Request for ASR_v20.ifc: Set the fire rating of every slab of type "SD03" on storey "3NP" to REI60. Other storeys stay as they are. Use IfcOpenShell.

First a look at what the model holds.

```python
import ifcopenshell
import ifcopenshell.util.element

model = ifcopenshell.open("ASR_v20.ifc")
print(model.schema)
storey = next(s for s in model.by_type("IfcBuildingStorey") if s.Name == "3NP")
slabs = [e for e in ifcopenshell.util.element.get_decomposition(storey) if e.is_a("IfcSlab")]
seen = {}
for e in slabs:
    element_type = ifcopenshell.util.element.get_type(e)
    key = (element_type.Name if element_type != e and element_type else None, ifcopenshell.util.element.get_pset(e, "Pset_SlabCommon", "FireRating"))
    seen[key] = seen.get(key, 0) + 1
for (name, value), count in sorted(seen.items(), key=str):
    print(count, "x", name, "|", value)
```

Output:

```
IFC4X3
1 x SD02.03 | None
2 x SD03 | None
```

```python
import ifcopenshell
import ifcopenshell.api.pset
import ifcopenshell.util.element

model = ifcopenshell.open("ASR_v20.ifc")

storey = next(s for s in model.by_type("IfcBuildingStorey") if s.Name == "3NP")
slabs = [e for e in ifcopenshell.util.element.get_decomposition(storey) if e.is_a("IfcSlab")]

count = 0
for e in slabs:
    element_type = ifcopenshell.util.element.get_type(e)
    if element_type in (None, e) or element_type.Name != "SD03":
        continue
    # add_pset returns the element's existing set when there is one.
    pset = ifcopenshell.api.pset.add_pset(model, product=e, name="Pset_SlabCommon")
    ifcopenshell.api.pset.edit_pset(model, pset=pset, properties={"FireRating": "REI60"})
    count += 1

print(count, "slabs updated")

model.write("ASR_v20_updated.ifc")
```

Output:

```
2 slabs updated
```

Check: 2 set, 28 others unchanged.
